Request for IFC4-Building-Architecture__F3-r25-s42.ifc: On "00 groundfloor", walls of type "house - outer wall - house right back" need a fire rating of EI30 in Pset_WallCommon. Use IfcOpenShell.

First a look at what the model holds.

```python
import ifcopenshell
import ifcopenshell.util.element

model = ifcopenshell.open("IFC4-Building-Architecture__F3-r25-s42.ifc")
print(model.schema)
storey = next(s for s in model.by_type("IfcBuildingStorey") if s.Name == "00 groundfloor")
walls = [e for e in ifcopenshell.util.element.get_decomposition(storey) if e.is_a("IfcWall")]
seen = {}
for e in walls:
    element_type = ifcopenshell.util.element.get_type(e)
    key = (element_type.Name if element_type != e and element_type else None, ifcopenshell.util.element.get_pset(e, "Pset_WallCommon", "FireRating"))
    seen[key] = seen.get(key, 0) + 1
for (name, value), count in sorted(seen.items(), key=str):
    print(count, "x", name, "|", value)
```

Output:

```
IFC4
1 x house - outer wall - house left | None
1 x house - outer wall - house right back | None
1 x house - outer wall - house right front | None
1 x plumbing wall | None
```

```python
import ifcopenshell
import ifcopenshell.api.pset
import ifcopenshell.util.element

model = ifcopenshell.open("IFC4-Building-Architecture__F3-r25-s42.ifc")

storey = next(s for s in model.by_type("IfcBuildingStorey") if s.Name == "00 groundfloor")
walls = [e for e in ifcopenshell.util.element.get_decomposition(storey) if e.is_a("IfcWall")]

count = 0
for e in walls:
    element_type = ifcopenshell.util.element.get_type(e)
    if element_type in (None, e) or element_type.Name != "house - outer wall - house right back":
        continue
    # add_pset returns the element's existing set when there is one.
    pset = ifcopenshell.api.pset.add_pset(model, product=e, name="Pset_WallCommon")
    ifcopenshell.api.pset.edit_pset(model, pset=pset, properties={"FireRating": "EI30"})
    count += 1

print(count, "walls updated")

model.write("IFC4-Building-Architecture__F3-r25-s42_updated.ifc")
```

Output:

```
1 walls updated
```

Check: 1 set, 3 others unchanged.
